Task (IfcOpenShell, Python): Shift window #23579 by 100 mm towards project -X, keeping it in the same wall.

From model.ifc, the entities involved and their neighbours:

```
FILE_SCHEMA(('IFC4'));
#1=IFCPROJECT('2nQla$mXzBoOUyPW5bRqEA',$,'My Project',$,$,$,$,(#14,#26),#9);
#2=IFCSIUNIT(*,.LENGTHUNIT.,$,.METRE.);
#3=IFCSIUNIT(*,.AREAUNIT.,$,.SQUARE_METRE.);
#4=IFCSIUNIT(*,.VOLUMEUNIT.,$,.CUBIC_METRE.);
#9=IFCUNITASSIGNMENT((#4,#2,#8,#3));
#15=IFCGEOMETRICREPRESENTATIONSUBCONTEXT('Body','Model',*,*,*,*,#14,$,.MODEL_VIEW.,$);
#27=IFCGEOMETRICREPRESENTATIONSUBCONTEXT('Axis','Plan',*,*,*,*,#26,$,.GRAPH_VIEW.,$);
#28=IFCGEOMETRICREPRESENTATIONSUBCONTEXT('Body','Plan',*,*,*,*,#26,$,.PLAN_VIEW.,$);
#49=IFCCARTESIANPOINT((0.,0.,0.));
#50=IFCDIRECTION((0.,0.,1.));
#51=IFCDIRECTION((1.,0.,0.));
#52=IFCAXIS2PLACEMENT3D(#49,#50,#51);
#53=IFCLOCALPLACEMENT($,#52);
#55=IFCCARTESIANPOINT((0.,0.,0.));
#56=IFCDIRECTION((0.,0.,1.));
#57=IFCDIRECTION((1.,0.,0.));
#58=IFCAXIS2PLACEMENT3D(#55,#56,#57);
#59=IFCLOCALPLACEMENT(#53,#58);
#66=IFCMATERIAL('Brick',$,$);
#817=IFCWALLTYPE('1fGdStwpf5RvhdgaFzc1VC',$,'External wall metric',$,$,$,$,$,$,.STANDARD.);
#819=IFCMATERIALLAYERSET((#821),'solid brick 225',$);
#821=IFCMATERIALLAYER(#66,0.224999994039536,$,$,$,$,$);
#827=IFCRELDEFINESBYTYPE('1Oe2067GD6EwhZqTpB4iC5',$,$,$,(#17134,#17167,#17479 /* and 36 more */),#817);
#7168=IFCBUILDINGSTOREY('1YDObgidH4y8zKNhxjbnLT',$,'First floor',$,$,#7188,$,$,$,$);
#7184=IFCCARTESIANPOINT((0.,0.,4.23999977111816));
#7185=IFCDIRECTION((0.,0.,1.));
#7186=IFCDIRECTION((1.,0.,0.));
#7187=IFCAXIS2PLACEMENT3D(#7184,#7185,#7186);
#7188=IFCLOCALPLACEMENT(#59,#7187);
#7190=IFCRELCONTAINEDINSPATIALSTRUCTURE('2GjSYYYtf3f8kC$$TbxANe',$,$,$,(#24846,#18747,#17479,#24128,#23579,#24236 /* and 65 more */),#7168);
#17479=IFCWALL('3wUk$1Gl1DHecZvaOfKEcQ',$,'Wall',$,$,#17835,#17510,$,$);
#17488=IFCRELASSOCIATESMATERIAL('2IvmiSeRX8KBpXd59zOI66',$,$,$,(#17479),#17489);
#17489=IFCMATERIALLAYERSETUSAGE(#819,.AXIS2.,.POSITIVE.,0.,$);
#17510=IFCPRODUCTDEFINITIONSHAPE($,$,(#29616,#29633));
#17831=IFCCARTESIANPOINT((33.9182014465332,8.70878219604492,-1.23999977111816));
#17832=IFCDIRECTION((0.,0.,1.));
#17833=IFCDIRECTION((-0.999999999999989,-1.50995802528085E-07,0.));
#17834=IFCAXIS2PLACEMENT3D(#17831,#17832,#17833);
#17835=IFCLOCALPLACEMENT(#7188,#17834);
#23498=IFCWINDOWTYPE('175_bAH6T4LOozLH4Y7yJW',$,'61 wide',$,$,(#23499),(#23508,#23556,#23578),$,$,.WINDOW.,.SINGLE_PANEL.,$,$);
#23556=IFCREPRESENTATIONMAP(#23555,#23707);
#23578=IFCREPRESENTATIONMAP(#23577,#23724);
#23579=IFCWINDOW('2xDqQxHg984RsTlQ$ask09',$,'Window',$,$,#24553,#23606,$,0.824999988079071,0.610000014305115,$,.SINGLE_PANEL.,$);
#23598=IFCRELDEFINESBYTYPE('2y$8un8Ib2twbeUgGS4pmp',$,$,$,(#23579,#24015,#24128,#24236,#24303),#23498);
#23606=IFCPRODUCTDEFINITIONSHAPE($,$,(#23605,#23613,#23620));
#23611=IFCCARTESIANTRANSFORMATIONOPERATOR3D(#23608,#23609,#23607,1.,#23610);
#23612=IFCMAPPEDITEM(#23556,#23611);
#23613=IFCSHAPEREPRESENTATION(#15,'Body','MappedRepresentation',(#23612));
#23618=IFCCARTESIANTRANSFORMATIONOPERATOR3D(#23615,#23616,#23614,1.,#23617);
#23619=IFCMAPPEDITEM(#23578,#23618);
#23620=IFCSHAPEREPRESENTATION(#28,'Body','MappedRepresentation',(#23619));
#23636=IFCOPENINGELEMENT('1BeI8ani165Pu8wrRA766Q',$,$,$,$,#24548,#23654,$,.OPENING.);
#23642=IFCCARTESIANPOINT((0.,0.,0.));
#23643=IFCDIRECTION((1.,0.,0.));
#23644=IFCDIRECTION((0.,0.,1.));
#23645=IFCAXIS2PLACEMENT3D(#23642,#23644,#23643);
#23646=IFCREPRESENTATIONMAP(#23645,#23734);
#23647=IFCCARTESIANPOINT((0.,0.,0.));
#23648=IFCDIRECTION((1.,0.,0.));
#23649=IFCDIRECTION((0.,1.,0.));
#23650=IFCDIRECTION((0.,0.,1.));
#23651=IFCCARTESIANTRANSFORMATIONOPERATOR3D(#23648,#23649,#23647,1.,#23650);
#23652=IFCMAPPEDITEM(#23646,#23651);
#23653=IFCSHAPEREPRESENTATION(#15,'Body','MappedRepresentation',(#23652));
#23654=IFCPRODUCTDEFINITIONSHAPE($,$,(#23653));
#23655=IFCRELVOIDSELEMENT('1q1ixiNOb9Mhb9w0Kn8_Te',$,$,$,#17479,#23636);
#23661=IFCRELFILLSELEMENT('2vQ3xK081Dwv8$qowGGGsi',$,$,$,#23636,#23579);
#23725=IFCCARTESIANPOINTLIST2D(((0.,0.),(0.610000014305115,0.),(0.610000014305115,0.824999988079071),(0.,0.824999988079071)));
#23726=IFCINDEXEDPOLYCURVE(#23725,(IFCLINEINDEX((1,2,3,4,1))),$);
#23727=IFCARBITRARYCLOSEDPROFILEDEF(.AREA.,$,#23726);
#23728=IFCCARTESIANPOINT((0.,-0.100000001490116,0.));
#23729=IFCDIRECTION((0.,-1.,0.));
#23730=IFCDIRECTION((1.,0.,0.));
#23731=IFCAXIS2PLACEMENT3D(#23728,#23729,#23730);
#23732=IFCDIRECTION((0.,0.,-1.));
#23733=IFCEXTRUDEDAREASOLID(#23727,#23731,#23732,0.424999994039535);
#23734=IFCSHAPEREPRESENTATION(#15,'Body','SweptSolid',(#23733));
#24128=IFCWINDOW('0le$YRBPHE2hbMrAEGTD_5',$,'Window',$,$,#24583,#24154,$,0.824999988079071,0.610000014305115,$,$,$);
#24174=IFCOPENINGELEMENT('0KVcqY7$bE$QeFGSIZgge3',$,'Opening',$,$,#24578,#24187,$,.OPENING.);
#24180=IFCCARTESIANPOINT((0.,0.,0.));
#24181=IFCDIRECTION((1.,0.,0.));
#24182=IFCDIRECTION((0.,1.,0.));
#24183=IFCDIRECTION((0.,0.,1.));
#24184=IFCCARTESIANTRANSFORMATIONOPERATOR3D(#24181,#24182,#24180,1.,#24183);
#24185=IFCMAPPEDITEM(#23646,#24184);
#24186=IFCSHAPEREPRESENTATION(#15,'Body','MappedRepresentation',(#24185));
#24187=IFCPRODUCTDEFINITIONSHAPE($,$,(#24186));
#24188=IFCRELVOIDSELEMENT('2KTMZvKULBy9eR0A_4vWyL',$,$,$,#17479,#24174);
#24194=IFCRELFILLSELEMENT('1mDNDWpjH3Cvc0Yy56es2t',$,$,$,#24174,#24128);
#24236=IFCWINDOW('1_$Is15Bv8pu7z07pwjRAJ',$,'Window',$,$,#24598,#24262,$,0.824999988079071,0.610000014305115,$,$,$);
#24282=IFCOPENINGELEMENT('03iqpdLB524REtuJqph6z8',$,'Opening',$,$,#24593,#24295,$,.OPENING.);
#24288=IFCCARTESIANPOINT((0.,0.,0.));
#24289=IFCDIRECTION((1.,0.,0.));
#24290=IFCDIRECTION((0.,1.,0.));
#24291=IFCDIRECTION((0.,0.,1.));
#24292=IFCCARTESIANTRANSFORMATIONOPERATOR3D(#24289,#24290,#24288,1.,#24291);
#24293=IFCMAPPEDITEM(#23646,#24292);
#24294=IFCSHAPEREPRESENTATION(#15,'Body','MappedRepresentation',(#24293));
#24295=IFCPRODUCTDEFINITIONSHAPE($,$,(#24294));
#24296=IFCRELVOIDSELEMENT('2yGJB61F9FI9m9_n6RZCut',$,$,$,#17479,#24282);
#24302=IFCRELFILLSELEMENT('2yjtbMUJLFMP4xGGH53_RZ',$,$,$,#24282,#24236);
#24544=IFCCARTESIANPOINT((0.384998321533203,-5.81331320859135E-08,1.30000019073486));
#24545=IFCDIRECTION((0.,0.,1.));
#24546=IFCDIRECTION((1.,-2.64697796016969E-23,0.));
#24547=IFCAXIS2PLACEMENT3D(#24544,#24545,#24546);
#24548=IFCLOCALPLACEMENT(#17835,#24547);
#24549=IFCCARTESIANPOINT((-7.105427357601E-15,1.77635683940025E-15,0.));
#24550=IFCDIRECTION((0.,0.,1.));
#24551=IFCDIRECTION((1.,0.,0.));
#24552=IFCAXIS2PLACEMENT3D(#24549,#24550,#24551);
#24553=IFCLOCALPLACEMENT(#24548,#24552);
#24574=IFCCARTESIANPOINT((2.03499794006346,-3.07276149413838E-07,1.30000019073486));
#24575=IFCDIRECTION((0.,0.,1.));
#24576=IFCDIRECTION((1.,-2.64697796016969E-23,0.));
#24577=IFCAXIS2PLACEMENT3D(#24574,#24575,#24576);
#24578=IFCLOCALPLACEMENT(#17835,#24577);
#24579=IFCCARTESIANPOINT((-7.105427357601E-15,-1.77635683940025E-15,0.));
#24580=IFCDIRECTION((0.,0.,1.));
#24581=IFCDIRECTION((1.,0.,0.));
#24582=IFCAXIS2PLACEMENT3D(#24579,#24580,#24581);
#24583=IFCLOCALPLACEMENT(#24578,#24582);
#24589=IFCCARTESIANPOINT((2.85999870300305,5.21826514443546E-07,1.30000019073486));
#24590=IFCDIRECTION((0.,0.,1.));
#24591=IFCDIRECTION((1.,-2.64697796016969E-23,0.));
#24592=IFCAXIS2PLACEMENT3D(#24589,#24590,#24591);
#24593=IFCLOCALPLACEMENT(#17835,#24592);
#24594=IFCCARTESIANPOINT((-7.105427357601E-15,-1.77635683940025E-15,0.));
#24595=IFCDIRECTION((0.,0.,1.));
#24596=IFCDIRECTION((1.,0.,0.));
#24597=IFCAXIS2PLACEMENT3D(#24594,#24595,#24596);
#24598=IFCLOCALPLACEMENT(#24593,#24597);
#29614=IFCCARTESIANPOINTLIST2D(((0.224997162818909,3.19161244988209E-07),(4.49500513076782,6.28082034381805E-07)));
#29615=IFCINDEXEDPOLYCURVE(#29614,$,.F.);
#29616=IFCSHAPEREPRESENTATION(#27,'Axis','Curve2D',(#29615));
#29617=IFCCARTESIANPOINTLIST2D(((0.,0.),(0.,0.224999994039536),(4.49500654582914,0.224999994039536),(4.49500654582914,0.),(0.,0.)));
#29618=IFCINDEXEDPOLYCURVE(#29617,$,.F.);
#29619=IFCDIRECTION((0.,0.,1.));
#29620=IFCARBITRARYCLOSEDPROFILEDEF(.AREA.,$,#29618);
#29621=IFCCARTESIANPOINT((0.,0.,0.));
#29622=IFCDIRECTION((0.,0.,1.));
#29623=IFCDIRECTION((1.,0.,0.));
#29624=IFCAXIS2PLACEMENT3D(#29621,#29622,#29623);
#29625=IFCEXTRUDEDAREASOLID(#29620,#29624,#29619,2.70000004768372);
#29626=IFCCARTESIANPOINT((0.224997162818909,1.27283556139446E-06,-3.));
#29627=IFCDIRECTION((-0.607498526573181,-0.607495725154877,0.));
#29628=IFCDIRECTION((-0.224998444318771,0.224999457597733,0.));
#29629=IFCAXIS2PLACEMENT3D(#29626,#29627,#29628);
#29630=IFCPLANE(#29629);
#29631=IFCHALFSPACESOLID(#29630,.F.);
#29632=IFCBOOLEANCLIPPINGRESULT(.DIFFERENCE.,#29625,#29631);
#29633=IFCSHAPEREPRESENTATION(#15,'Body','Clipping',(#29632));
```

```python
import ifcopenshell
import ifcopenshell.api.geometry
import ifcopenshell.util.placement
import ifcopenshell.util.unit

model = ifcopenshell.open("model.ifc")
unit_scale = ifcopenshell.util.unit.calculate_unit_scale(model)

window = model.by_guid("2xDqQxHg984RsTlQ$ask09")
opening = window.FillsVoids[0].RelatingOpeningElement
wall = opening.VoidsElements[0].RelatingBuildingElement

wall_matrix = ifcopenshell.util.placement.get_local_placement(wall.ObjectPlacement)
shift = wall_matrix[:3, 0] * 0.1 / unit_scale
before = ifcopenshell.util.placement.get_local_placement(window.ObjectPlacement)[:3, 3].copy()

# The window is placed relative to its opening, so it follows when the opening moves.
matrix = ifcopenshell.util.placement.get_local_placement(opening.ObjectPlacement)
matrix[:3, 3] += shift
ifcopenshell.api.geometry.edit_object_placement(
    model, product=opening, matrix=matrix, is_si=False, should_transform_children=True
)

after = ifcopenshell.util.placement.get_local_placement(window.ObjectPlacement)[:3, 3]
print("window moved by", (after - before).round(3) + 0.0)

model.write("model-out.ifc")
```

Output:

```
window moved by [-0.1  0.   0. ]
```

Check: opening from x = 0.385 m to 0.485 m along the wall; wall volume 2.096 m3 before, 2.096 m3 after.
